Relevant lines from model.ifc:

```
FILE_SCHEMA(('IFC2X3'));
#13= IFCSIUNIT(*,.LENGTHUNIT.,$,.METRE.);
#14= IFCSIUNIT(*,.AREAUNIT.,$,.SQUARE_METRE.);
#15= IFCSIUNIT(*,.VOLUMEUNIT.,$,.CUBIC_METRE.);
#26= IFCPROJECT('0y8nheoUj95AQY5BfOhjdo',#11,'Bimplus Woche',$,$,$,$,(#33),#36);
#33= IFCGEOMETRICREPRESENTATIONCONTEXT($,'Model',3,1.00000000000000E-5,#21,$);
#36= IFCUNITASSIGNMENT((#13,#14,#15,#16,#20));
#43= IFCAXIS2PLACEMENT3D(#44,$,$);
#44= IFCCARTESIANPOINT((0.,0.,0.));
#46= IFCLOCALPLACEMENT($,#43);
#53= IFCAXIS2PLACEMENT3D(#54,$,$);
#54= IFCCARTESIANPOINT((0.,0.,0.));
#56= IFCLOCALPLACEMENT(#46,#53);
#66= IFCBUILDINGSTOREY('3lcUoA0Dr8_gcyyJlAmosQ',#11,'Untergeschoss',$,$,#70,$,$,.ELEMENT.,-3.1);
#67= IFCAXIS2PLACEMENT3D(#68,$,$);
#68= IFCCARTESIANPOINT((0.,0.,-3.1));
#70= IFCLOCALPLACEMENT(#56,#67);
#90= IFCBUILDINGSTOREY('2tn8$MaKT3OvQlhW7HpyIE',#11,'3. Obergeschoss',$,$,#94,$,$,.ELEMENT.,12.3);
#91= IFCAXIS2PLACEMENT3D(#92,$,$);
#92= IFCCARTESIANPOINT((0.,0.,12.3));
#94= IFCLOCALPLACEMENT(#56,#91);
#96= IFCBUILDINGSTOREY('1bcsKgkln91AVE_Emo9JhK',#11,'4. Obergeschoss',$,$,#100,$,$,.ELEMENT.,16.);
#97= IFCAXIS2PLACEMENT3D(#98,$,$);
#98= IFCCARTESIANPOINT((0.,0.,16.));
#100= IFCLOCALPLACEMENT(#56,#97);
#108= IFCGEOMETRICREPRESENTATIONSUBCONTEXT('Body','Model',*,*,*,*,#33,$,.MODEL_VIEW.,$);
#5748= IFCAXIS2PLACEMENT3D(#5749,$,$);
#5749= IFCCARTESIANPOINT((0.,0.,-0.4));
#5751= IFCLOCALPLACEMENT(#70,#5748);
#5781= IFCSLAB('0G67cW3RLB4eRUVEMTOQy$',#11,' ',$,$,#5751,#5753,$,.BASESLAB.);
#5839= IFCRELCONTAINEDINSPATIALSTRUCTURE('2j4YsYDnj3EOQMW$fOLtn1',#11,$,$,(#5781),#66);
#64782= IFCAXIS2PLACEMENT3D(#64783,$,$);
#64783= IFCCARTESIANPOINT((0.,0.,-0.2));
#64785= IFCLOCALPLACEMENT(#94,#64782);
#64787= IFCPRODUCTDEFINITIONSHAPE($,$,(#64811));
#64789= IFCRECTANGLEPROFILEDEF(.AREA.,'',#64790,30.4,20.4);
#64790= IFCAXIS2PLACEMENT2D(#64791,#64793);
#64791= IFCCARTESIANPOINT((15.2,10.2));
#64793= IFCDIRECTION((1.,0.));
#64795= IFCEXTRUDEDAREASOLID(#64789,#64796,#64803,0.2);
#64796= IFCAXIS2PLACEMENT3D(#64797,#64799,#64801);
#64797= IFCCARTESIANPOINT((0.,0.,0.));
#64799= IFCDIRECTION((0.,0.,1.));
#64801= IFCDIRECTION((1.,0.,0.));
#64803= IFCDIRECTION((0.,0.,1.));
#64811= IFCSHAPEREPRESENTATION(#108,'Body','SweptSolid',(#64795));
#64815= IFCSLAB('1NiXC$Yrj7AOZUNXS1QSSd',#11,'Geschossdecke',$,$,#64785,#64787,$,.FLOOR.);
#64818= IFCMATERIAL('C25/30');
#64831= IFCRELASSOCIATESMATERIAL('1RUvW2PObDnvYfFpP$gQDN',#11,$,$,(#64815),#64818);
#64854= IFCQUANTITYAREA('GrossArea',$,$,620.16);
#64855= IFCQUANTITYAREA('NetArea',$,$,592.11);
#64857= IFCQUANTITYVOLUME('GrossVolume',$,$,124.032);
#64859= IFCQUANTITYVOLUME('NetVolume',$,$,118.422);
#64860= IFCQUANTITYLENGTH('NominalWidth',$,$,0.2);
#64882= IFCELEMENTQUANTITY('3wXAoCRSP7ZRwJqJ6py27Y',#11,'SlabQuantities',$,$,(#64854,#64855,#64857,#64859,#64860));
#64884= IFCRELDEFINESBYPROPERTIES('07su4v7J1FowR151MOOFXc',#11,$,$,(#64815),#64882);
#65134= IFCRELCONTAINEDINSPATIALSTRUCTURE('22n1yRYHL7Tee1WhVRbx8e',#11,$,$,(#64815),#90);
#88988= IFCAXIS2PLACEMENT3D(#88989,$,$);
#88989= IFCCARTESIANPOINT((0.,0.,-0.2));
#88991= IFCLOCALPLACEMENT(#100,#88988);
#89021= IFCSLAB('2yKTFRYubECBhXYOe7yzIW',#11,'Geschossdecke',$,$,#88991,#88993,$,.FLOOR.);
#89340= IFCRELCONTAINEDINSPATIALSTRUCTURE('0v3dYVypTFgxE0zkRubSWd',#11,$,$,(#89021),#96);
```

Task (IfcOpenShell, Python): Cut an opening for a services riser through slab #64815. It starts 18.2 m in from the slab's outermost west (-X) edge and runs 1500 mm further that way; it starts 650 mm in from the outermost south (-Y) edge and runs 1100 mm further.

```python
import numpy as np
import ifcopenshell
import ifcopenshell.api.feature
import ifcopenshell.api.geometry
import ifcopenshell.api.pset
import ifcopenshell.api.root
import ifcopenshell.geom
import ifcopenshell.util.element
import ifcopenshell.util.placement
import ifcopenshell.util.representation
import ifcopenshell.util.shape
import ifcopenshell.util.unit

model = ifcopenshell.open("model.ifc")
unit_scale = ifcopenshell.util.unit.calculate_unit_scale(model)
area_scale = ifcopenshell.util.unit.calculate_unit_scale(model, "AREAUNIT")
volume_scale = ifcopenshell.util.unit.calculate_unit_scale(model, "VOLUMEUNIT")
settings = ifcopenshell.geom.settings()


def volume(element):
    """Net volume in cubic metres, openings subtracted."""
    shape = ifcopenshell.geom.create_shape(settings, element)
    return ifcopenshell.util.shape.get_volume(shape.geometry)


slab = model.by_guid("1NiXC$Yrj7AOZUNXS1QSSd")
before = volume(slab)

# Extent in the slab's own axes, in metres. The edges named are its -X and -Y sides.
slab_shape = ifcopenshell.geom.create_shape(settings, slab)
vertices = ifcopenshell.util.shape.get_vertices(slab_shape.geometry)
x_min, y_min, bottom = vertices.min(axis=0)
top = vertices[:, 2].max()

opening = ifcopenshell.api.root.create_entity(model, ifc_class="IfcOpeningElement", name="Services riser opening")
context = ifcopenshell.util.representation.get_context(model, "Model", "Body", "MODEL_VIEW")
width, depth = 1.5, 1.1
outline = [(0.0, 0.0), (width, 0.0), (width, depth), (0.0, depth), (0.0, 0.0)]
# Overshoot both faces by 50 mm so the cut is clean.
shape = ifcopenshell.api.geometry.add_slab_representation(
    model, context=context, depth=top - bottom + 0.1, polyline=outline
)
ifcopenshell.api.geometry.assign_representation(model, product=opening, representation=shape)

matrix = ifcopenshell.util.placement.get_local_placement(slab.ObjectPlacement)
matrix[:, 3] = matrix @ np.append(np.array([x_min + 18.2, y_min + 0.65, bottom - 0.05]) / unit_scale, 1.0)
ifcopenshell.api.geometry.edit_object_placement(model, product=opening, matrix=matrix, is_si=False)
ifcopenshell.api.feature.add_feature(model, feature=opening, element=slab)

after = volume(slab)

# Update the slab's stored quantities.
qto = model.by_id(ifcopenshell.util.element.get_pset(slab, "SlabQuantities", should_inherit=False)["id"])
ifcopenshell.api.pset.edit_qto(model, qto=qto, properties={
    "NetArea": after / (top - bottom) / area_scale,
    "NetVolume": after / volume_scale,
})

print(f"slab volume {before:.3f} -> {after:.3f} m3")

model.write("model_edited.ifc")
```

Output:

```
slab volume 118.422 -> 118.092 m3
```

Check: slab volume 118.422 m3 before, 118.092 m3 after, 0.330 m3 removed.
